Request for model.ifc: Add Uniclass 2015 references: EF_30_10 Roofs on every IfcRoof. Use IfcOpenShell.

First a look at what the model holds.

```python
import ifcopenshell

model = ifcopenshell.open("model.ifc")
print(model.schema)
print("classifications:", [c.Name for c in model.by_type("IfcClassification")])
for ifc_class in ("IfcDoor", "IfcRoof", "IfcStair", "IfcWall", "IfcWindow"):
    print(ifc_class, len(model.by_type(ifc_class)))
```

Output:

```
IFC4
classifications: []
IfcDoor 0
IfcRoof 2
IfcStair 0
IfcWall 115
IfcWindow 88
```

```python
import ifcopenshell
import ifcopenshell.api.classification

model = ifcopenshell.open("model.ifc")

system = ifcopenshell.api.classification.add_classification(model, classification="Uniclass 2015")

codes = {
    "IfcRoof": ("EF_30_10", "Roofs"),
}
for ifc_class, (code, name) in codes.items():
    products = model.by_type(ifc_class)
    ifcopenshell.api.classification.add_reference(
        model, products=products, classification=system, identification=code, name=name
    )
    print(code, len(products))

model.write("model_updated.ifc")
```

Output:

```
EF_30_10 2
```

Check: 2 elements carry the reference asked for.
